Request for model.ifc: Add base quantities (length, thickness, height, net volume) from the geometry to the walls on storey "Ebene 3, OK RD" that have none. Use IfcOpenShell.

First a look at what the model holds.

```python
import ifcopenshell
import ifcopenshell.util.element
import ifcopenshell.util.unit

model = ifcopenshell.open("model.ifc")
print(model.schema)
for unit_type in ("LENGTHUNIT", "AREAUNIT", "VOLUMEUNIT"):
    print(unit_type, ifcopenshell.util.unit.calculate_unit_scale(model, unit_type))
storey = next(s for s in model.by_type("IfcBuildingStorey") if s.Name == "Ebene 3, OK RD")
walls = [e for e in ifcopenshell.util.element.get_decomposition(storey) if e.is_a("IfcWall")]
for e in sorted(walls, key=lambda e: e.id()):
    print(e.id(), e.is_a(), e.Name, list(ifcopenshell.util.element.get_psets(e, qtos_only=True)), sep=" | ")
```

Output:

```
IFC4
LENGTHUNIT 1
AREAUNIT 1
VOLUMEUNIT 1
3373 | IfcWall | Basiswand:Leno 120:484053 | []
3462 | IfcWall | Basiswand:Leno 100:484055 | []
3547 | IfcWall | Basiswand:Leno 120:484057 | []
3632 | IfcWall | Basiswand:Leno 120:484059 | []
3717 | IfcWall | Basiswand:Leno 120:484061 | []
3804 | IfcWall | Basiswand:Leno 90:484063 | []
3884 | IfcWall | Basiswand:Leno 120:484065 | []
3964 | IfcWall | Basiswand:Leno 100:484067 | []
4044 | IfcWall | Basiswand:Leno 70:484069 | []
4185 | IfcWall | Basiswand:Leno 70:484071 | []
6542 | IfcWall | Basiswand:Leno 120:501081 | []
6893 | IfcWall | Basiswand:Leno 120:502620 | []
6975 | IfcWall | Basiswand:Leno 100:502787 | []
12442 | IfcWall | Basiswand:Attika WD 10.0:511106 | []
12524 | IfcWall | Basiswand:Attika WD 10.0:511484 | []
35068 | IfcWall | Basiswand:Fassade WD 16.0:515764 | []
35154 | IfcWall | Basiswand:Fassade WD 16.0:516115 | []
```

```python
import ifcopenshell
import ifcopenshell.api.pset
import ifcopenshell.geom
import ifcopenshell.util.element
import ifcopenshell.util.shape
import ifcopenshell.util.unit

model = ifcopenshell.open("model.ifc")
unit_scale = ifcopenshell.util.unit.calculate_unit_scale(model)
volume_scale = ifcopenshell.util.unit.calculate_unit_scale(model, "VOLUMEUNIT")
settings = ifcopenshell.geom.settings()

storey = next(s for s in model.by_type("IfcBuildingStorey") if s.Name == "Ebene 3, OK RD")
walls = [e for e in ifcopenshell.util.element.get_decomposition(storey) if e.is_a("IfcWall")]

for e in sorted(walls, key=lambda e: e.id()):
    if ifcopenshell.util.element.get_psets(e, qtos_only=True, should_inherit=False):
        continue
    # Geometry comes back in metres, in the element's own axes.
    shape = ifcopenshell.geom.create_shape(settings, e)
    values = {
        "Length": ifcopenshell.util.shape.get_x(shape.geometry) / unit_scale,
        "Width": ifcopenshell.util.shape.get_y(shape.geometry) / unit_scale,
        "Height": ifcopenshell.util.shape.get_z(shape.geometry) / unit_scale,
        "NetVolume": ifcopenshell.util.shape.get_volume(shape.geometry) / volume_scale,
    }
    qto = ifcopenshell.api.pset.add_qto(model, product=e, name="Qto_WallBaseQuantities")
    ifcopenshell.api.pset.edit_qto(model, qto=qto, properties=values)
    print(e.id(), {k: round(v, 3) for k, v in values.items()})

model.write("model_edited.ifc")
```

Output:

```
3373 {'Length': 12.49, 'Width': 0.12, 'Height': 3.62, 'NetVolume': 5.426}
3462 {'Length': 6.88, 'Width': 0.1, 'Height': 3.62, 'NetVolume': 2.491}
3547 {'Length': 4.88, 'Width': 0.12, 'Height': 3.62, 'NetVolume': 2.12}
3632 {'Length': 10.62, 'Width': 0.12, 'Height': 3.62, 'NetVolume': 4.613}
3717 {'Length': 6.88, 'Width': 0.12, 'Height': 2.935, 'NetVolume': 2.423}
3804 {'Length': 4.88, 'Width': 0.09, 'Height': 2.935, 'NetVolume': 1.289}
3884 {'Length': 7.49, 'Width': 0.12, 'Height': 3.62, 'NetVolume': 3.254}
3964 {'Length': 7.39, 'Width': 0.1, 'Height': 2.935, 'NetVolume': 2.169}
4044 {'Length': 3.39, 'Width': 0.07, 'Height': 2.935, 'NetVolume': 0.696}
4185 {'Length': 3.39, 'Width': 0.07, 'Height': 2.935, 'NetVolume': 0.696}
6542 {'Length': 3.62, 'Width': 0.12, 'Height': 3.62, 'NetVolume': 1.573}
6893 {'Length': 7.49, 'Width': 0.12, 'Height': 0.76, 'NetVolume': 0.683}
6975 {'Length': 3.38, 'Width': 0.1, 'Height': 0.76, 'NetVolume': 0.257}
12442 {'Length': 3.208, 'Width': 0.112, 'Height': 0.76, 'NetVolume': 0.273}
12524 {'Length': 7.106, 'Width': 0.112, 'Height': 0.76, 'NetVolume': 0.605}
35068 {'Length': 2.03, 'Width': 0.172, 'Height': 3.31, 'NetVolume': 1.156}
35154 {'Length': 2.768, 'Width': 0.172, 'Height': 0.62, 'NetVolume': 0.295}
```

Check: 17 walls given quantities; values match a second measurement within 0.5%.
